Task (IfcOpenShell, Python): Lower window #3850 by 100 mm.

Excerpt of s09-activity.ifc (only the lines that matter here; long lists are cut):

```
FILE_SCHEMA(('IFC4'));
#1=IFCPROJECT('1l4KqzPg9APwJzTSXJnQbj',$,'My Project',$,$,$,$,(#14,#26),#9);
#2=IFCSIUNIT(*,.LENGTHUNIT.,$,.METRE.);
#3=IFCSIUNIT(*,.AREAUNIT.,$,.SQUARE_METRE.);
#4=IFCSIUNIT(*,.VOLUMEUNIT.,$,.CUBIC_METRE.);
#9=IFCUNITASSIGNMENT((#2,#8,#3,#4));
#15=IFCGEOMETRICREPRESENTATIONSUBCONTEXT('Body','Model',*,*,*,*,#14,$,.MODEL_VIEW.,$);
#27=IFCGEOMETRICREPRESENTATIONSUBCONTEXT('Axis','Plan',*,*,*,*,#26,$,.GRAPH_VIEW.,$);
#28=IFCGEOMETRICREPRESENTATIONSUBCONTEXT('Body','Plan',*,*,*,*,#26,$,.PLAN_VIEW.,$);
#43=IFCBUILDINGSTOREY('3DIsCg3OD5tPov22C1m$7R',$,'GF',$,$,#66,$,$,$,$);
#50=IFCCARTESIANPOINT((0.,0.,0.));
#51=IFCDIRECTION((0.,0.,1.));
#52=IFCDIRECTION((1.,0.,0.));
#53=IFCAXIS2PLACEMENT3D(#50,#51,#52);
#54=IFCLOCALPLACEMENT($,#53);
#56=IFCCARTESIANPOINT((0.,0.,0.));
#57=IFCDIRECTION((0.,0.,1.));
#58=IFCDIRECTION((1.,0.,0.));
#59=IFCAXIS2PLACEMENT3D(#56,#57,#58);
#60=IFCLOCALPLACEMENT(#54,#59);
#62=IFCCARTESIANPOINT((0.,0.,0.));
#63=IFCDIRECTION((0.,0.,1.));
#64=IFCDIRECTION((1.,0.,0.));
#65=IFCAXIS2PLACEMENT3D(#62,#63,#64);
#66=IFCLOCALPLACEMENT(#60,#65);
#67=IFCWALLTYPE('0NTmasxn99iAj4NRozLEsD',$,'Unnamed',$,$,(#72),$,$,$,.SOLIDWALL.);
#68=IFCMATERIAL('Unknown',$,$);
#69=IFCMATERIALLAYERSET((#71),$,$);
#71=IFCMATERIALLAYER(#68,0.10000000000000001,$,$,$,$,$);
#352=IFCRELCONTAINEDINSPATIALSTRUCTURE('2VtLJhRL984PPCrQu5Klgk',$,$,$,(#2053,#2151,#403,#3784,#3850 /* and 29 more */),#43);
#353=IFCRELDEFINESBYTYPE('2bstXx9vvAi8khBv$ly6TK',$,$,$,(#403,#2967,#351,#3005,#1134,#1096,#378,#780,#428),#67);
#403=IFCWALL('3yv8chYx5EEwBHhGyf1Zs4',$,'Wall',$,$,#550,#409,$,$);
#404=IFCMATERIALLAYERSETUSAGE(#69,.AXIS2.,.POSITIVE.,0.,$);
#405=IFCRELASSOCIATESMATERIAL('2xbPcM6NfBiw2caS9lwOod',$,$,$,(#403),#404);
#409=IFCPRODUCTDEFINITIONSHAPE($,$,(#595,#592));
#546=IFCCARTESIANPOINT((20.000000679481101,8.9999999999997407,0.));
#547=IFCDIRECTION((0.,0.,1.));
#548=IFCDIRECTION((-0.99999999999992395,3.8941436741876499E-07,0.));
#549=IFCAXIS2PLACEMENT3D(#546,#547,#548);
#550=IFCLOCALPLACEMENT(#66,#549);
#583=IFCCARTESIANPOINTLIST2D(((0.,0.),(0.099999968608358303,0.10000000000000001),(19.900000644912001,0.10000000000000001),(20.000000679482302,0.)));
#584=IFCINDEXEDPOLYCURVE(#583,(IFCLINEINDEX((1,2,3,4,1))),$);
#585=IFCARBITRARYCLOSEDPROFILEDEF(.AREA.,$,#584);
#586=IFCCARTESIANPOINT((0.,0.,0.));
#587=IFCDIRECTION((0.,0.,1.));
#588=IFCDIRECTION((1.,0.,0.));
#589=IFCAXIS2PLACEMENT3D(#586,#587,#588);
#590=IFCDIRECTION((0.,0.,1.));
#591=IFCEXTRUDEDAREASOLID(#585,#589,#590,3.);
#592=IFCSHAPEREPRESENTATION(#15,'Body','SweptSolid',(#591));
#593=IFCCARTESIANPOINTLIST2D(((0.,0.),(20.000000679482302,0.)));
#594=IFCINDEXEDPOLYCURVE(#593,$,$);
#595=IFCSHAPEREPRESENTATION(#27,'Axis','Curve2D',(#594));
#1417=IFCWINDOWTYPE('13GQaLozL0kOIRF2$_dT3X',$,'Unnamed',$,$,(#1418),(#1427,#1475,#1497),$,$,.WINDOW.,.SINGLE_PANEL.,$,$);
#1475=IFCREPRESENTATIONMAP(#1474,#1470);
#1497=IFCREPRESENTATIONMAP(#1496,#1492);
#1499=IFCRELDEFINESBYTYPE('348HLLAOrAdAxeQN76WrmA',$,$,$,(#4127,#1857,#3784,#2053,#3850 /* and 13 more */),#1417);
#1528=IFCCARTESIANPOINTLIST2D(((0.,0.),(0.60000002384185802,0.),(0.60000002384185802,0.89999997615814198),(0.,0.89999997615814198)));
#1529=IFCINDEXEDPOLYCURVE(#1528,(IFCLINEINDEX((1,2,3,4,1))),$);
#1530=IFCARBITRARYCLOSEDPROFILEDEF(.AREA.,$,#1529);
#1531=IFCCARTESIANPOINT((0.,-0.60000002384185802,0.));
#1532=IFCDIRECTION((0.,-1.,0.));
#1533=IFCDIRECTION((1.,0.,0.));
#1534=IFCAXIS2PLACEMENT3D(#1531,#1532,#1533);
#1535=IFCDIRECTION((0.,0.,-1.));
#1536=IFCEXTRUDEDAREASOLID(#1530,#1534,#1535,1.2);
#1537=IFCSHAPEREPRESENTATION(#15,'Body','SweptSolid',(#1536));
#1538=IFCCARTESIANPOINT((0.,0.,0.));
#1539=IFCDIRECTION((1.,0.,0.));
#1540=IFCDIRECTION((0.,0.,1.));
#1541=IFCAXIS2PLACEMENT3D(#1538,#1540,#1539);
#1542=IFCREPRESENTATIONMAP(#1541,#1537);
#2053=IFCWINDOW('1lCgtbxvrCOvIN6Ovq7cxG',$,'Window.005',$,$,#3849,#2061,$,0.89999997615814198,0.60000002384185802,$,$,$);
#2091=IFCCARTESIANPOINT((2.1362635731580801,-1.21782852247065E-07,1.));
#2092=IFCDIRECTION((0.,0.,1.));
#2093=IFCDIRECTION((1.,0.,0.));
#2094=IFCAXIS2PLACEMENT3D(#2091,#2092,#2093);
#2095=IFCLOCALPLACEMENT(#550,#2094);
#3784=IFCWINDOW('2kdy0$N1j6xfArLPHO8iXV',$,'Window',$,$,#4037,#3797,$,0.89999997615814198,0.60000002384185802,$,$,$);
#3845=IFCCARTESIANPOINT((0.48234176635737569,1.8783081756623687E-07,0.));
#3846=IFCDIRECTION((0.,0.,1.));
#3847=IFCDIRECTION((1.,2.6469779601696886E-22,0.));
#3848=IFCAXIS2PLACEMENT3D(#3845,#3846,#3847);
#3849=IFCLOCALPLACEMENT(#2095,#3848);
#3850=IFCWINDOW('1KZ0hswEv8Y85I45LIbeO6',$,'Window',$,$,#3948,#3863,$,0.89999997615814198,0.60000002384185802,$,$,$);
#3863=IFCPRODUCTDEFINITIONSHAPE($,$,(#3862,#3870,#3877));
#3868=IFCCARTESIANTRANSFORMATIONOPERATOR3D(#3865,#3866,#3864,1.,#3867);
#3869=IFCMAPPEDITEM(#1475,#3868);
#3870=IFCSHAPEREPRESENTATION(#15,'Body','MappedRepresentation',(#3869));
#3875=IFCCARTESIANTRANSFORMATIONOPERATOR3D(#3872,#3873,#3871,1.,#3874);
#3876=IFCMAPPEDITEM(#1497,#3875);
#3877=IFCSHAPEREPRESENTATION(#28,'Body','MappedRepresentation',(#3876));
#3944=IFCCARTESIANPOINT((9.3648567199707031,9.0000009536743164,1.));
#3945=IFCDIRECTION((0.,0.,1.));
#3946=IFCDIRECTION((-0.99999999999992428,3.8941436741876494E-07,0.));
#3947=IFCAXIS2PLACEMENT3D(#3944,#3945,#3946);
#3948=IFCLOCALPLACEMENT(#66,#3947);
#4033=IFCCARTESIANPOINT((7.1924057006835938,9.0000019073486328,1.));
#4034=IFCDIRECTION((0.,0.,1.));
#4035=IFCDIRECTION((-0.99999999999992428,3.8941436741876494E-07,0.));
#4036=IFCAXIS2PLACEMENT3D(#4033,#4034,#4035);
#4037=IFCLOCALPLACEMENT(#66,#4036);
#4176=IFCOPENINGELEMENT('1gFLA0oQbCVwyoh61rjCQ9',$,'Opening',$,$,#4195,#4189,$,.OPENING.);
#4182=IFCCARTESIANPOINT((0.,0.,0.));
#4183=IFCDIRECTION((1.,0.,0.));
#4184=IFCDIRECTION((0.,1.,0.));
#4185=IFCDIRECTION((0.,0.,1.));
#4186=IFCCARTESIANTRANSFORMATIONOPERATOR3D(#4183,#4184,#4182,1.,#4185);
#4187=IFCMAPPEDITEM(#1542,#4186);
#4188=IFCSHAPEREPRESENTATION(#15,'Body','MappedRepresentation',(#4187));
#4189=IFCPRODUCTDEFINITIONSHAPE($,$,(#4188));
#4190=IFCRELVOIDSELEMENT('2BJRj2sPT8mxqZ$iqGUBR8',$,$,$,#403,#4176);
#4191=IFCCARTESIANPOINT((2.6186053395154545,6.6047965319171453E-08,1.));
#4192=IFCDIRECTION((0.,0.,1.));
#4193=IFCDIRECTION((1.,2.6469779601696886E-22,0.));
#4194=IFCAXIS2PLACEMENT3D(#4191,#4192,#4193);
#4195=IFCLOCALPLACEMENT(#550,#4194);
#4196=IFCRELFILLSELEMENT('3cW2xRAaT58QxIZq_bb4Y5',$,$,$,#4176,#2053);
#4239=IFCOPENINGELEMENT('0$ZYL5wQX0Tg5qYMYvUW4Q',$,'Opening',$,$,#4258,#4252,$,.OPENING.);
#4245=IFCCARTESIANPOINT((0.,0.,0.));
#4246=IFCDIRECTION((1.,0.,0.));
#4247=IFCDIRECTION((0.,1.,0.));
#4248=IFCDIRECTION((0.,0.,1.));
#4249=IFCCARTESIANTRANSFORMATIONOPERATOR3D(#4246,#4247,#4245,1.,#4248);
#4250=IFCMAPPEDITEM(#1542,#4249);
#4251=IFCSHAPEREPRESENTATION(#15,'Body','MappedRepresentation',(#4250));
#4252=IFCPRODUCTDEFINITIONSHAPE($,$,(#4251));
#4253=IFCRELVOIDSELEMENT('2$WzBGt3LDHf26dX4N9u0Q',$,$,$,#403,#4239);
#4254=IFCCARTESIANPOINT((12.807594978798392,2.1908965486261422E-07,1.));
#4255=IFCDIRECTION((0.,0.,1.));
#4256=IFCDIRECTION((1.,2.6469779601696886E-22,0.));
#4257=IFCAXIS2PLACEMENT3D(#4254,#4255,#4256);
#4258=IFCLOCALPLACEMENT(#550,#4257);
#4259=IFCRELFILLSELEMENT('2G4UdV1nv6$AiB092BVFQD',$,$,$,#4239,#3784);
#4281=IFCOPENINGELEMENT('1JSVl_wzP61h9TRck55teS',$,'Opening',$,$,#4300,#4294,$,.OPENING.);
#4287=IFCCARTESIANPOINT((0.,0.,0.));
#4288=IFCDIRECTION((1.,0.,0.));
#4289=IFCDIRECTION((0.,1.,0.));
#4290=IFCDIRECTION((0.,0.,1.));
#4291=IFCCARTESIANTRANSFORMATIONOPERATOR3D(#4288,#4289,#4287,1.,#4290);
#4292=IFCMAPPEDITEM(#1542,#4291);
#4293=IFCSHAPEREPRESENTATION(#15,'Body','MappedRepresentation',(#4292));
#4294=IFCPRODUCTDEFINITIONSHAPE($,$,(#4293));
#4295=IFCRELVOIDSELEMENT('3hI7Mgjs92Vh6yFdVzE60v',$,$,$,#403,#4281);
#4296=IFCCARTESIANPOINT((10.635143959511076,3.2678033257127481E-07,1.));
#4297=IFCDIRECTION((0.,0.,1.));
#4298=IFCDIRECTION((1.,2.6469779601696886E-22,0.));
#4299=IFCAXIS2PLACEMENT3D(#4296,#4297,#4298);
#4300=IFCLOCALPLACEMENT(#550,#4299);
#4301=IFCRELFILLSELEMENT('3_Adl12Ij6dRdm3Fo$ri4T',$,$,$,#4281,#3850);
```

```python
import numpy as np
import ifcopenshell
import ifcopenshell.api.geometry
import ifcopenshell.util.placement
import ifcopenshell.util.unit

model = ifcopenshell.open("s09-activity.ifc")
unit_scale = ifcopenshell.util.unit.calculate_unit_scale(model)

window = model.by_guid("1KZ0hswEv8Y85I45LIbeO6")
opening = window.FillsVoids[0].RelatingOpeningElement
dz = -0.1 / unit_scale

shift = np.array([0.0, 0.0, dz])
# The window is not placed relative to its opening, so move both.
for product in (opening, window):
    matrix = ifcopenshell.util.placement.get_local_placement(product.ObjectPlacement)
    matrix[:3, 3] += shift
    ifcopenshell.api.geometry.edit_object_placement(model, product=product, matrix=matrix, is_si=False)

print(f"moved by {dz * unit_scale:+.3f} m")

model.write("s09-activity_v2.ifc")
```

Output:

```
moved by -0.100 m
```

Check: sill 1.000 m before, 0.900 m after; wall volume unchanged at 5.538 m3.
